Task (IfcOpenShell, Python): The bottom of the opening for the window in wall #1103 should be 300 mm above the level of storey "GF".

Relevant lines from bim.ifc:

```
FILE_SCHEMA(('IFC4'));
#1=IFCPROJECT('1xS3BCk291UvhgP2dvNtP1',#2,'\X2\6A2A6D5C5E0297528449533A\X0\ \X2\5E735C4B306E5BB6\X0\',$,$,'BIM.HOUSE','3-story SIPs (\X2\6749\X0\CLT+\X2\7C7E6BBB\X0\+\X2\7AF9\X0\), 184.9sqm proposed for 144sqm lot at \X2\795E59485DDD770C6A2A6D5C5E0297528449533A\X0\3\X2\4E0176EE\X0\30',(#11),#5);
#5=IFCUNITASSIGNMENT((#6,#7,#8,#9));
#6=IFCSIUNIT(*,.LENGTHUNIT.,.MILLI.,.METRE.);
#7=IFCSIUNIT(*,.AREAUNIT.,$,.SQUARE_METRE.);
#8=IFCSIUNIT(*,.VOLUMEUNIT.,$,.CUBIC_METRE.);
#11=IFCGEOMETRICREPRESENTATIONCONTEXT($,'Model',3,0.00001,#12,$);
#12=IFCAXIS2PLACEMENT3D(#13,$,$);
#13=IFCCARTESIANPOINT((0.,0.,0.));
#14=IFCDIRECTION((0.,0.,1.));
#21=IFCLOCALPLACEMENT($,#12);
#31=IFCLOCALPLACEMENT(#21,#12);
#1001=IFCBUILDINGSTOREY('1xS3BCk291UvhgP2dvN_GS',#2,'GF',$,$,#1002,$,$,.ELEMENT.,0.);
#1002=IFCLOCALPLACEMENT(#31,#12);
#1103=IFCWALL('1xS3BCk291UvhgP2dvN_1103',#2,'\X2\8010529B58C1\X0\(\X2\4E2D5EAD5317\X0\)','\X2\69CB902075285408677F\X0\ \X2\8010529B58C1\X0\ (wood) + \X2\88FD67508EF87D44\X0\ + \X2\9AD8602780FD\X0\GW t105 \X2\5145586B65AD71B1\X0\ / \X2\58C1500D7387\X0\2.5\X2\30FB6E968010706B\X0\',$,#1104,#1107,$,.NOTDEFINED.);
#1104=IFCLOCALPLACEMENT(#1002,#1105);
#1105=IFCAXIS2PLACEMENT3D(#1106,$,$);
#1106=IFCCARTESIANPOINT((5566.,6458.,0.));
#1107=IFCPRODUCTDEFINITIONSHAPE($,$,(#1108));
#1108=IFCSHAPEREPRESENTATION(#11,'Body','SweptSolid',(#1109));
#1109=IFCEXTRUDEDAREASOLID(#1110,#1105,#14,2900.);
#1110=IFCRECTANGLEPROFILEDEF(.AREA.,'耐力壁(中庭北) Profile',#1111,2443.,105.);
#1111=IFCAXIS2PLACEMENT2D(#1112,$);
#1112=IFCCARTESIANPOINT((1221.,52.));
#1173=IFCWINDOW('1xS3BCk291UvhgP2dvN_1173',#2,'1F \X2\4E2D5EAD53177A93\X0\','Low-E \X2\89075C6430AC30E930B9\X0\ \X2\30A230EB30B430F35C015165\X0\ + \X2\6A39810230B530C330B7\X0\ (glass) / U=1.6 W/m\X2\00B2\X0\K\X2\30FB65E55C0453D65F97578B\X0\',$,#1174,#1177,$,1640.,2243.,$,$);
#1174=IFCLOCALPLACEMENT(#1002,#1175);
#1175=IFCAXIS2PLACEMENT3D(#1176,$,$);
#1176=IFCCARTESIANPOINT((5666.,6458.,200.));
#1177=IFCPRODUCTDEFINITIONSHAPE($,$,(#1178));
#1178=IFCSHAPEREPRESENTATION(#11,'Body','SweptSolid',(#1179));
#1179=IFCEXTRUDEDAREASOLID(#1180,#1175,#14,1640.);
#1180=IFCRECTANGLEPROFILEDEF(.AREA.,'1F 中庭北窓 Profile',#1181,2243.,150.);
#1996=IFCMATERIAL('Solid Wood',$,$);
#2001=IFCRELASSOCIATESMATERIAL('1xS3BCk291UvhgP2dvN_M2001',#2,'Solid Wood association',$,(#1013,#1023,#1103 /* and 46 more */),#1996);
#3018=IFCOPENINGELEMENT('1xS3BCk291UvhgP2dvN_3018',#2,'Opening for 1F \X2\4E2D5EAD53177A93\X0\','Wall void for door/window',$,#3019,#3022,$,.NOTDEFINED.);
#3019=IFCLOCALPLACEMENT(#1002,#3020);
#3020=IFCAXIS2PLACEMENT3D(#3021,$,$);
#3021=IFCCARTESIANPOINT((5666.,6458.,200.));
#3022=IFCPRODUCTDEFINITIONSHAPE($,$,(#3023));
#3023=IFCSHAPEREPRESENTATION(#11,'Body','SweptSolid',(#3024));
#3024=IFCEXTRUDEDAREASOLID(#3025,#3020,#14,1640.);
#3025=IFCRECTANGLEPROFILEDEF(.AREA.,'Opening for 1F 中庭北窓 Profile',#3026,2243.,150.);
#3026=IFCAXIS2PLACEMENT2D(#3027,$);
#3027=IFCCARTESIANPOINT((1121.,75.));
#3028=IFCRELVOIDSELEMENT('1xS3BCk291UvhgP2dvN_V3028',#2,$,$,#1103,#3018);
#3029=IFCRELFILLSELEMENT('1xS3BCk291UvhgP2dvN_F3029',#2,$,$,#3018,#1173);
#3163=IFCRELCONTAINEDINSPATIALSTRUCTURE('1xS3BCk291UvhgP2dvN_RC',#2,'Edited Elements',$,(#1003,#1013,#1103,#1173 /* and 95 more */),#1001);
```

```python
import numpy as np
import ifcopenshell
import ifcopenshell.api.geometry
import ifcopenshell.geom
import ifcopenshell.util.element
import ifcopenshell.util.placement
import ifcopenshell.util.shape
import ifcopenshell.util.unit

model = ifcopenshell.open("bim.ifc")
unit_scale = ifcopenshell.util.unit.calculate_unit_scale(model)

window = model.by_guid("1xS3BCk291UvhgP2dvN_1173")
opening = window.FillsVoids[0].RelatingOpeningElement
storey = ifcopenshell.util.element.get_container(window, ifc_class="IfcBuildingStorey")
level = ifcopenshell.util.placement.get_local_placement(storey.ObjectPlacement)[2, 3]

# The opening's origin need not be at the sill, so measure its lowest point.
shape = ifcopenshell.geom.create_shape(ifcopenshell.geom.settings(), opening)
bottom = ifcopenshell.util.shape.get_shape_bottom_elevation(shape, shape.geometry) / unit_scale
dz = level + 0.3 / unit_scale - bottom

shift = np.array([0.0, 0.0, dz])
# The window is not placed relative to its opening, so move both.
for product in (opening, window):
    matrix = ifcopenshell.util.placement.get_local_placement(product.ObjectPlacement)
    matrix[:3, 3] += shift
    ifcopenshell.api.geometry.edit_object_placement(model, product=product, matrix=matrix, is_si=False)

print(f"moved by {dz * unit_scale:+.3f} m")

model.write("bim-out.ifc")
```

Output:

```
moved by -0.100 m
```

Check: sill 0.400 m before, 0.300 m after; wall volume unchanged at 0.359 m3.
